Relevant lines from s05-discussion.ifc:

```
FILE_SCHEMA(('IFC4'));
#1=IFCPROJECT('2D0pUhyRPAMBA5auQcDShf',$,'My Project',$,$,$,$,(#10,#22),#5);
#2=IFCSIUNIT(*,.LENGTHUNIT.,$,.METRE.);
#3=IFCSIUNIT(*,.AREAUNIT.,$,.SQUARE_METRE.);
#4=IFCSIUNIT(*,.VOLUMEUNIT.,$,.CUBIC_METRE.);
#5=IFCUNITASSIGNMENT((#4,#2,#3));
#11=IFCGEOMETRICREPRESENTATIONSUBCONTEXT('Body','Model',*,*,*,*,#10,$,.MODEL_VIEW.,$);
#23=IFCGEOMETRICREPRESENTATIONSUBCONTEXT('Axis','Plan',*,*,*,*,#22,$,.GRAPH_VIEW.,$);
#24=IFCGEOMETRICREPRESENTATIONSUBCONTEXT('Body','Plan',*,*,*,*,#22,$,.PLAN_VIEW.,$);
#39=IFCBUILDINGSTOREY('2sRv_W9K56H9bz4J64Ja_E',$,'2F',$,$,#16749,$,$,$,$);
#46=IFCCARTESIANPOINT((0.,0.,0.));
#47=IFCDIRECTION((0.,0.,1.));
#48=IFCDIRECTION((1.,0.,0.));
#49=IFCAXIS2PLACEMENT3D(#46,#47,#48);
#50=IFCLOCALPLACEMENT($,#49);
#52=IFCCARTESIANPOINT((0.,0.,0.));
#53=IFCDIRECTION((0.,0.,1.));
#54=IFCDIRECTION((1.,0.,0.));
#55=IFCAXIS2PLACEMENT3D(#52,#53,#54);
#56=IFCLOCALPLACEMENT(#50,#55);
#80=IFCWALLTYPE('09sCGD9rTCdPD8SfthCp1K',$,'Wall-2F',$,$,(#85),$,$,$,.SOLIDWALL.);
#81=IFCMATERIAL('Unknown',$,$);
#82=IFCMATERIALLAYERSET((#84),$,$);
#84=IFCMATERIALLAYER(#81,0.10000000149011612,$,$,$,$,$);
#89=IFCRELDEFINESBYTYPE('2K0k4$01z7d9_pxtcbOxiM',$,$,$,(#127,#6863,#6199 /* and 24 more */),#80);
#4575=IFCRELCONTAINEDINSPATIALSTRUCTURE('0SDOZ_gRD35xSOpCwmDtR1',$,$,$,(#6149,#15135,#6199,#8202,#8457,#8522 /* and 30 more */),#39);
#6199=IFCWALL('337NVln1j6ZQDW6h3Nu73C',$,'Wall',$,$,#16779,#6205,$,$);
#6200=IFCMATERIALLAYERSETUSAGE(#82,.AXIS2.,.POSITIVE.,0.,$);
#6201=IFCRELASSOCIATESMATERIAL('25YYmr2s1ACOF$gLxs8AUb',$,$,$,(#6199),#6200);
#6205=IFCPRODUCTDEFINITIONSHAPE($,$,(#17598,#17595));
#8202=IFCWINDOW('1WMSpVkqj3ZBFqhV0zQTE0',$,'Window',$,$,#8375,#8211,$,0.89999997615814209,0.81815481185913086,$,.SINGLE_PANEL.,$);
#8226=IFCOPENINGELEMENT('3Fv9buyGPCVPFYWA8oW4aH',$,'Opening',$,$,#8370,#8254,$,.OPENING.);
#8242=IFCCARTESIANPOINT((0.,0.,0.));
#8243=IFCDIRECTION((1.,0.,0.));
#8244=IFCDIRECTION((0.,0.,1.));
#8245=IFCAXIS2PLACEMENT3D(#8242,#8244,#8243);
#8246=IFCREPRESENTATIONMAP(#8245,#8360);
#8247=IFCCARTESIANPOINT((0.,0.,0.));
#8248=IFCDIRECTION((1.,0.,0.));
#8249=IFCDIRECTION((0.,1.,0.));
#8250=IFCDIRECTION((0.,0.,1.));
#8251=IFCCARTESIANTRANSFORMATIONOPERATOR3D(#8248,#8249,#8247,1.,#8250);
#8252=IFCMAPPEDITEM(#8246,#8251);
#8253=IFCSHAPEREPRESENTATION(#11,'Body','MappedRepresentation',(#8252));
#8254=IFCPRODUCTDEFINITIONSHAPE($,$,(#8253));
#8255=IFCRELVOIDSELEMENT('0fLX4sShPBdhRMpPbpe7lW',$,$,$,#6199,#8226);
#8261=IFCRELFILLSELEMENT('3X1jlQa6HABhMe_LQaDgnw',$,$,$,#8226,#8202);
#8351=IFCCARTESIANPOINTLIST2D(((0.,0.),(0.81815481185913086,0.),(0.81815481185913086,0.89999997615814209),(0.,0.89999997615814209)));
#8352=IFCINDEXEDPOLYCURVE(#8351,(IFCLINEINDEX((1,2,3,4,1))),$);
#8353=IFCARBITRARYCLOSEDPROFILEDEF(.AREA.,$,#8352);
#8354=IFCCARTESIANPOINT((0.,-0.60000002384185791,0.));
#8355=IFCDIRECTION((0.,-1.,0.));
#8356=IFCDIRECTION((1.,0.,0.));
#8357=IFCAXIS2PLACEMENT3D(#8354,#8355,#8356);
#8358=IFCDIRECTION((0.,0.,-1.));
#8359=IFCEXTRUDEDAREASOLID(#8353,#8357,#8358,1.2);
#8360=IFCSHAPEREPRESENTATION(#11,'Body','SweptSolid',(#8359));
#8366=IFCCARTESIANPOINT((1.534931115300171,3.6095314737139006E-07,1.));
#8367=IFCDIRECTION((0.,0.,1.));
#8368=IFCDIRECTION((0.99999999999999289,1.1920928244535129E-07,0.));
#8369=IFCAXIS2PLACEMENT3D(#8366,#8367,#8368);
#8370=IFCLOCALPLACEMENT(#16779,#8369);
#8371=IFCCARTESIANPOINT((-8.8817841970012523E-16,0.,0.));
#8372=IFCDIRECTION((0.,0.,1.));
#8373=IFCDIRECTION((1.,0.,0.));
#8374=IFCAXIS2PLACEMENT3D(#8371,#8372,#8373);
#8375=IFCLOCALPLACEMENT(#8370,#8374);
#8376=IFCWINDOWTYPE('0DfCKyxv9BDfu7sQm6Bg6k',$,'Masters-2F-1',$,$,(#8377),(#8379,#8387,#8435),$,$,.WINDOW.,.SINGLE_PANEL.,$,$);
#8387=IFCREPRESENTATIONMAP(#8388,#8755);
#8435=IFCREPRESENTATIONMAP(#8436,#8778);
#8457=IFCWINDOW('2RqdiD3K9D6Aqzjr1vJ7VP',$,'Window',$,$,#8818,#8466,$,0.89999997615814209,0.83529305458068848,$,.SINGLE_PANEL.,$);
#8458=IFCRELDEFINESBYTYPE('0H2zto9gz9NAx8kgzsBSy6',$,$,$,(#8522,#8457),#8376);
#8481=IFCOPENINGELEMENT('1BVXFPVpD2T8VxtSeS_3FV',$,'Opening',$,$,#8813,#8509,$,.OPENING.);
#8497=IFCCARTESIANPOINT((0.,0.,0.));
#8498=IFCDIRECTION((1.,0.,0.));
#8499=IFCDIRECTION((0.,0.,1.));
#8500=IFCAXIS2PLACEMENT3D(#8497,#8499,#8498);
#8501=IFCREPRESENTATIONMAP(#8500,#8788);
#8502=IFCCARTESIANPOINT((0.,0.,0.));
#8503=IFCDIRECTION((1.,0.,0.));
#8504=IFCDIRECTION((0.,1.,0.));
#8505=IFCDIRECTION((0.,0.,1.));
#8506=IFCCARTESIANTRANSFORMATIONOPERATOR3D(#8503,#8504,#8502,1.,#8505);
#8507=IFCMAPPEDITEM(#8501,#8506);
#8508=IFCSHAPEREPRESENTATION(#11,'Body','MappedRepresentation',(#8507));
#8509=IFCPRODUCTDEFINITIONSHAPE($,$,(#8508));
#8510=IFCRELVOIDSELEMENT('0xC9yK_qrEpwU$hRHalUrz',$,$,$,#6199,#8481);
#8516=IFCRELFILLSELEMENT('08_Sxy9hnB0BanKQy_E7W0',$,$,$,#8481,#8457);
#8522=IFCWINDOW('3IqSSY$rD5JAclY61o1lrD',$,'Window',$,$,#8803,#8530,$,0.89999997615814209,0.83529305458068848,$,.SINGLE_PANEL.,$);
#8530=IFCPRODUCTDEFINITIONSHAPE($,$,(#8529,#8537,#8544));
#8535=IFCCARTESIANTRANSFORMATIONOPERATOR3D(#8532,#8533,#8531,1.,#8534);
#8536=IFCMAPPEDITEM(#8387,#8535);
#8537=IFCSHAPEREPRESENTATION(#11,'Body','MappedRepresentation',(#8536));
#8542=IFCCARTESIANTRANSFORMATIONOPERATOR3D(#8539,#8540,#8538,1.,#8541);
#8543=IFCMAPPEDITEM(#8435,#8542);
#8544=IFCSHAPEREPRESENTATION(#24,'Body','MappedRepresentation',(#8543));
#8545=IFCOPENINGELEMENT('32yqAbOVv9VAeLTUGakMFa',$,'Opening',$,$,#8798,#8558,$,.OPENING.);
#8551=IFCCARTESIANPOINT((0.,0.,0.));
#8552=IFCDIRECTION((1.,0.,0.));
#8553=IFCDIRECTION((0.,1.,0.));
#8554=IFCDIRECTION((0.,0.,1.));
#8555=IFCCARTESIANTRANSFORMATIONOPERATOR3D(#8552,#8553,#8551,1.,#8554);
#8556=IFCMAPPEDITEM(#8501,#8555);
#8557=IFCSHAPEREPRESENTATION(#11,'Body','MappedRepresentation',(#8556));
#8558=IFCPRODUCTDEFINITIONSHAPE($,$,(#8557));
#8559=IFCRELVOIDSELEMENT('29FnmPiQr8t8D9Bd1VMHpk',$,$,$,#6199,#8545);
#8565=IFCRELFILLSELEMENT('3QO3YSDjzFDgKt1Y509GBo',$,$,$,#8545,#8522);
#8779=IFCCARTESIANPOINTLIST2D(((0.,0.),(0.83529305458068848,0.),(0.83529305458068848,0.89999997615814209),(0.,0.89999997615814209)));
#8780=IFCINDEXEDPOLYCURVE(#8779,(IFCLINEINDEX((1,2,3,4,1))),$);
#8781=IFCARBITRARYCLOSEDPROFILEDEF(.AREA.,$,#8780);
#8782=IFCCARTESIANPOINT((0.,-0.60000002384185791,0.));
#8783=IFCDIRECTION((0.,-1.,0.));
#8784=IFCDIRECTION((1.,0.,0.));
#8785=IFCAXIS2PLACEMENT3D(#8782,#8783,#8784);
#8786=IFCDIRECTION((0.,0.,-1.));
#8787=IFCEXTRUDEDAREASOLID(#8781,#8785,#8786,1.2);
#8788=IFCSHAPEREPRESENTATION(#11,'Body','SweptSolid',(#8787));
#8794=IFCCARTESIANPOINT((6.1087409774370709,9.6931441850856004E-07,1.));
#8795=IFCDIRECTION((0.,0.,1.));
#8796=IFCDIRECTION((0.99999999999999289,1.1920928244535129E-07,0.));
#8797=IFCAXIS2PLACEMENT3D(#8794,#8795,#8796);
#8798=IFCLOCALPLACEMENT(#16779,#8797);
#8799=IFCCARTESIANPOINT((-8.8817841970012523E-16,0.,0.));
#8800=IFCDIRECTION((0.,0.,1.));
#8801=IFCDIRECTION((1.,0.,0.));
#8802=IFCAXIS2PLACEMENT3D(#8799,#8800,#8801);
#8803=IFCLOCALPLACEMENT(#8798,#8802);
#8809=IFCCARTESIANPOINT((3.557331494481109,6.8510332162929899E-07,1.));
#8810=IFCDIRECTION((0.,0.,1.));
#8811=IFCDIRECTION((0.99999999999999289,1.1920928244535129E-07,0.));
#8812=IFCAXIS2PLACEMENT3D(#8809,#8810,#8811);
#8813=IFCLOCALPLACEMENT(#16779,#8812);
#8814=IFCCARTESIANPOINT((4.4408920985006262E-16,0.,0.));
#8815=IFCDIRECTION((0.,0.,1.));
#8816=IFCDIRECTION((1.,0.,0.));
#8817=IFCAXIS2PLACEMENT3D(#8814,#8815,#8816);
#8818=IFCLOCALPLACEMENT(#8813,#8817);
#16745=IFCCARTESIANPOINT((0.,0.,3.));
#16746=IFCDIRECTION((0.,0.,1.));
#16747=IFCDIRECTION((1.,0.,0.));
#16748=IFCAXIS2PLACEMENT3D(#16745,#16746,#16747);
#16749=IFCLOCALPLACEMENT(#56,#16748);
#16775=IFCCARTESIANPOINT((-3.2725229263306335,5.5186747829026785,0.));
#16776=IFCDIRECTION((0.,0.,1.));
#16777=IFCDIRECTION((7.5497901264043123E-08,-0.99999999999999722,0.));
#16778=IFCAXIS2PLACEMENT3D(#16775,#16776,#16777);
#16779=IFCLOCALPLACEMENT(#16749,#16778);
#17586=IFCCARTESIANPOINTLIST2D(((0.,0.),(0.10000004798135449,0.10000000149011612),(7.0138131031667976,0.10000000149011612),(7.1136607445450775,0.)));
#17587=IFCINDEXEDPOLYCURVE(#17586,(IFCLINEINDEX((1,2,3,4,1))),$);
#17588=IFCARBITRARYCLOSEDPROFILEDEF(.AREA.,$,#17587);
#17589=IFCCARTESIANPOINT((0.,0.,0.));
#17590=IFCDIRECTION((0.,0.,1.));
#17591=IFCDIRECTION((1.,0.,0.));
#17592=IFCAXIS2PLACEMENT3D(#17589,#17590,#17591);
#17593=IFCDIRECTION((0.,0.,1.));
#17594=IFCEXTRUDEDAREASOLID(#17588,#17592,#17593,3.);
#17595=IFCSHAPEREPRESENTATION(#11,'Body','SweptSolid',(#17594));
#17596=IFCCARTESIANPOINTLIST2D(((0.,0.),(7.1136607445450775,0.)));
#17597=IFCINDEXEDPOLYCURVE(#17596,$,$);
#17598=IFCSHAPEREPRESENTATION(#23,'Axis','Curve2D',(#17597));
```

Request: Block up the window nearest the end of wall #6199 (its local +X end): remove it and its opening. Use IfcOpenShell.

```python
import ifcopenshell
import ifcopenshell.api.feature
import ifcopenshell.api.root
import ifcopenshell.geom
import ifcopenshell.util.shape

model = ifcopenshell.open("s05-discussion.ifc")
settings = ifcopenshell.geom.settings()


def volume(element):
    """Net volume in cubic metres, openings subtracted."""
    shape = ifcopenshell.geom.create_shape(settings, element)
    return ifcopenshell.util.shape.get_volume(shape.geometry)


window = model.by_id(8522)
opening = window.FillsVoids[0].RelatingOpeningElement
wall = opening.VoidsElements[0].RelatingBuildingElement
before = volume(wall)

ifcopenshell.api.root.remove_product(model, product=window)
ifcopenshell.api.feature.remove_feature(model, feature=opening)

after = volume(wall)

print(f"wall volume {before:.3f} -> {after:.3f} m3")

model.write("s05-discussion-out.ifc")
```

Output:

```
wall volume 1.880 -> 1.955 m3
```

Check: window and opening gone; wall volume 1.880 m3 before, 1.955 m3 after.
